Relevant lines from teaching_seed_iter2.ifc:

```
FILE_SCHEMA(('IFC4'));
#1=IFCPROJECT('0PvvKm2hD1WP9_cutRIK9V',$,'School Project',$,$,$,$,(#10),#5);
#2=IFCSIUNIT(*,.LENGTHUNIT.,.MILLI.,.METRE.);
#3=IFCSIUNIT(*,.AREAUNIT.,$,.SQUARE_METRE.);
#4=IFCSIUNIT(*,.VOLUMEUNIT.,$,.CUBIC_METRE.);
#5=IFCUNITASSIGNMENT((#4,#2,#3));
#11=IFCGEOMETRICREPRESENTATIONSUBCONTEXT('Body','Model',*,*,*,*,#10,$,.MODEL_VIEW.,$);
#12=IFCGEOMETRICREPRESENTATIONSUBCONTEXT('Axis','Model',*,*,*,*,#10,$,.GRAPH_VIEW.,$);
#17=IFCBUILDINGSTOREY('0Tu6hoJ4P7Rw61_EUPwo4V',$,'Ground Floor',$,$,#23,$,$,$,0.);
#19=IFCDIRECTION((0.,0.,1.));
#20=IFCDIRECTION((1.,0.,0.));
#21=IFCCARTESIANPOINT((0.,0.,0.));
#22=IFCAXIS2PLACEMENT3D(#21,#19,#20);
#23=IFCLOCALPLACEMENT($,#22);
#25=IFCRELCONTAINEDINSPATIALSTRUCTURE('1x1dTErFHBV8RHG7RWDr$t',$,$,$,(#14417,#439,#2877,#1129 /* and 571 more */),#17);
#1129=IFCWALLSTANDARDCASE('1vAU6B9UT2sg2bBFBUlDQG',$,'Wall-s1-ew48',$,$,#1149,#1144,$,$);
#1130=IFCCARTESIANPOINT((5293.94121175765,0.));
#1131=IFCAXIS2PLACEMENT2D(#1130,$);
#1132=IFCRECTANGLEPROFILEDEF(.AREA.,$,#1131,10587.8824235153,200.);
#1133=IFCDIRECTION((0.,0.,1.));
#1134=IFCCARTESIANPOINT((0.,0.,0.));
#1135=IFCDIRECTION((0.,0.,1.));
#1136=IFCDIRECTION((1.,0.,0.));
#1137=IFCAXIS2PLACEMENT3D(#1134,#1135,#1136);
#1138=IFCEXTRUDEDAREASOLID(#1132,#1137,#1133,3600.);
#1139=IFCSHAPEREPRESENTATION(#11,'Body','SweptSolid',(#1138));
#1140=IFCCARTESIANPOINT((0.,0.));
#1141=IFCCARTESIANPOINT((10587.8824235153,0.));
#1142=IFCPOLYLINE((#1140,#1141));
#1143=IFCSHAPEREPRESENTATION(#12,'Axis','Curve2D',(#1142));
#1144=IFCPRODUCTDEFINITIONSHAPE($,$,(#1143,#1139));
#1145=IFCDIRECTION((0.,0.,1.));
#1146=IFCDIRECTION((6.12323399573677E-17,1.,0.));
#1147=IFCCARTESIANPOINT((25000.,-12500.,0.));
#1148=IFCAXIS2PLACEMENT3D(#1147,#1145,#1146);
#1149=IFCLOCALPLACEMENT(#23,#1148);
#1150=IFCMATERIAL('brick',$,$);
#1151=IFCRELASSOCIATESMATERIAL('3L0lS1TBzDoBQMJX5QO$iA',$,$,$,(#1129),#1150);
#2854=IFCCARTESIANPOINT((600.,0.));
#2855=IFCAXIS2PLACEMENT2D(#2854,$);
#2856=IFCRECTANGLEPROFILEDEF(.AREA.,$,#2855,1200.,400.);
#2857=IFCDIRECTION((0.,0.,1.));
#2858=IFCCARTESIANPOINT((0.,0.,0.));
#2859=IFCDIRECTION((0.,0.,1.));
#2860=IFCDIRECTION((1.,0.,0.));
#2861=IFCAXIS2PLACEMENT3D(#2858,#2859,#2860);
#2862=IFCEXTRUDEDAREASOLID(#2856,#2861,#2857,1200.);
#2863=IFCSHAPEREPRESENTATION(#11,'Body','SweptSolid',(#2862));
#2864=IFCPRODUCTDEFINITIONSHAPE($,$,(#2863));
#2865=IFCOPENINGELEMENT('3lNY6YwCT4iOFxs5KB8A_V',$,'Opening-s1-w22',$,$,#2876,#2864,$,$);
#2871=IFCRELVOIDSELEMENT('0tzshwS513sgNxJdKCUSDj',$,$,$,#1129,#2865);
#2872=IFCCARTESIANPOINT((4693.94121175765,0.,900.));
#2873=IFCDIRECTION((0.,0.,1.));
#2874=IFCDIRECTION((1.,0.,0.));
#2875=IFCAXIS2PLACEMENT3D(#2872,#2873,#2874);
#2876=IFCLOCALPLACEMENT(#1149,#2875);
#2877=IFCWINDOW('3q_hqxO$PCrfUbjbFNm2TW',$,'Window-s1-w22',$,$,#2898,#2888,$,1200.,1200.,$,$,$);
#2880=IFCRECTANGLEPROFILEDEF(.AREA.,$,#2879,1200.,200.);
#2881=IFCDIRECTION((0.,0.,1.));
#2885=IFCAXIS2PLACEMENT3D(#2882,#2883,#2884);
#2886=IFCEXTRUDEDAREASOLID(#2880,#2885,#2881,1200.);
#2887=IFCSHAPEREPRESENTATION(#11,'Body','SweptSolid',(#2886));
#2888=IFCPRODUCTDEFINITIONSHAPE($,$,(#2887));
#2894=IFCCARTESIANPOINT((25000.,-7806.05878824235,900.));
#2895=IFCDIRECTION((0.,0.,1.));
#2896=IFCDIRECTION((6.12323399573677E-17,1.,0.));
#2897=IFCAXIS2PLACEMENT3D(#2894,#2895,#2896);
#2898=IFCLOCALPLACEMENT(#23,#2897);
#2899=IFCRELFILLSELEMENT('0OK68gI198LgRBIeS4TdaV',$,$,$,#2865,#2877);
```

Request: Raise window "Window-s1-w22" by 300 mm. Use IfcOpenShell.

```python
import numpy as np
import ifcopenshell
import ifcopenshell.api.geometry
import ifcopenshell.util.placement
import ifcopenshell.util.unit

model = ifcopenshell.open("teaching_seed_iter2.ifc")
unit_scale = ifcopenshell.util.unit.calculate_unit_scale(model)

window = model.by_guid("3q_hqxO$PCrfUbjbFNm2TW")
opening = window.FillsVoids[0].RelatingOpeningElement
dz = 0.3 / unit_scale

shift = np.array([0.0, 0.0, dz])
# The window is not placed relative to its opening, so move both.
for product in (opening, window):
    matrix = ifcopenshell.util.placement.get_local_placement(product.ObjectPlacement)
    matrix[:3, 3] += shift
    ifcopenshell.api.geometry.edit_object_placement(model, product=product, matrix=matrix, is_si=False)

print(f"moved by {dz * unit_scale:+.3f} m")

model.write("teaching_seed_iter2_edited.ifc")
```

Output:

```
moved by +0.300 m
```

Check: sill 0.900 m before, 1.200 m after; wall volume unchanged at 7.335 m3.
